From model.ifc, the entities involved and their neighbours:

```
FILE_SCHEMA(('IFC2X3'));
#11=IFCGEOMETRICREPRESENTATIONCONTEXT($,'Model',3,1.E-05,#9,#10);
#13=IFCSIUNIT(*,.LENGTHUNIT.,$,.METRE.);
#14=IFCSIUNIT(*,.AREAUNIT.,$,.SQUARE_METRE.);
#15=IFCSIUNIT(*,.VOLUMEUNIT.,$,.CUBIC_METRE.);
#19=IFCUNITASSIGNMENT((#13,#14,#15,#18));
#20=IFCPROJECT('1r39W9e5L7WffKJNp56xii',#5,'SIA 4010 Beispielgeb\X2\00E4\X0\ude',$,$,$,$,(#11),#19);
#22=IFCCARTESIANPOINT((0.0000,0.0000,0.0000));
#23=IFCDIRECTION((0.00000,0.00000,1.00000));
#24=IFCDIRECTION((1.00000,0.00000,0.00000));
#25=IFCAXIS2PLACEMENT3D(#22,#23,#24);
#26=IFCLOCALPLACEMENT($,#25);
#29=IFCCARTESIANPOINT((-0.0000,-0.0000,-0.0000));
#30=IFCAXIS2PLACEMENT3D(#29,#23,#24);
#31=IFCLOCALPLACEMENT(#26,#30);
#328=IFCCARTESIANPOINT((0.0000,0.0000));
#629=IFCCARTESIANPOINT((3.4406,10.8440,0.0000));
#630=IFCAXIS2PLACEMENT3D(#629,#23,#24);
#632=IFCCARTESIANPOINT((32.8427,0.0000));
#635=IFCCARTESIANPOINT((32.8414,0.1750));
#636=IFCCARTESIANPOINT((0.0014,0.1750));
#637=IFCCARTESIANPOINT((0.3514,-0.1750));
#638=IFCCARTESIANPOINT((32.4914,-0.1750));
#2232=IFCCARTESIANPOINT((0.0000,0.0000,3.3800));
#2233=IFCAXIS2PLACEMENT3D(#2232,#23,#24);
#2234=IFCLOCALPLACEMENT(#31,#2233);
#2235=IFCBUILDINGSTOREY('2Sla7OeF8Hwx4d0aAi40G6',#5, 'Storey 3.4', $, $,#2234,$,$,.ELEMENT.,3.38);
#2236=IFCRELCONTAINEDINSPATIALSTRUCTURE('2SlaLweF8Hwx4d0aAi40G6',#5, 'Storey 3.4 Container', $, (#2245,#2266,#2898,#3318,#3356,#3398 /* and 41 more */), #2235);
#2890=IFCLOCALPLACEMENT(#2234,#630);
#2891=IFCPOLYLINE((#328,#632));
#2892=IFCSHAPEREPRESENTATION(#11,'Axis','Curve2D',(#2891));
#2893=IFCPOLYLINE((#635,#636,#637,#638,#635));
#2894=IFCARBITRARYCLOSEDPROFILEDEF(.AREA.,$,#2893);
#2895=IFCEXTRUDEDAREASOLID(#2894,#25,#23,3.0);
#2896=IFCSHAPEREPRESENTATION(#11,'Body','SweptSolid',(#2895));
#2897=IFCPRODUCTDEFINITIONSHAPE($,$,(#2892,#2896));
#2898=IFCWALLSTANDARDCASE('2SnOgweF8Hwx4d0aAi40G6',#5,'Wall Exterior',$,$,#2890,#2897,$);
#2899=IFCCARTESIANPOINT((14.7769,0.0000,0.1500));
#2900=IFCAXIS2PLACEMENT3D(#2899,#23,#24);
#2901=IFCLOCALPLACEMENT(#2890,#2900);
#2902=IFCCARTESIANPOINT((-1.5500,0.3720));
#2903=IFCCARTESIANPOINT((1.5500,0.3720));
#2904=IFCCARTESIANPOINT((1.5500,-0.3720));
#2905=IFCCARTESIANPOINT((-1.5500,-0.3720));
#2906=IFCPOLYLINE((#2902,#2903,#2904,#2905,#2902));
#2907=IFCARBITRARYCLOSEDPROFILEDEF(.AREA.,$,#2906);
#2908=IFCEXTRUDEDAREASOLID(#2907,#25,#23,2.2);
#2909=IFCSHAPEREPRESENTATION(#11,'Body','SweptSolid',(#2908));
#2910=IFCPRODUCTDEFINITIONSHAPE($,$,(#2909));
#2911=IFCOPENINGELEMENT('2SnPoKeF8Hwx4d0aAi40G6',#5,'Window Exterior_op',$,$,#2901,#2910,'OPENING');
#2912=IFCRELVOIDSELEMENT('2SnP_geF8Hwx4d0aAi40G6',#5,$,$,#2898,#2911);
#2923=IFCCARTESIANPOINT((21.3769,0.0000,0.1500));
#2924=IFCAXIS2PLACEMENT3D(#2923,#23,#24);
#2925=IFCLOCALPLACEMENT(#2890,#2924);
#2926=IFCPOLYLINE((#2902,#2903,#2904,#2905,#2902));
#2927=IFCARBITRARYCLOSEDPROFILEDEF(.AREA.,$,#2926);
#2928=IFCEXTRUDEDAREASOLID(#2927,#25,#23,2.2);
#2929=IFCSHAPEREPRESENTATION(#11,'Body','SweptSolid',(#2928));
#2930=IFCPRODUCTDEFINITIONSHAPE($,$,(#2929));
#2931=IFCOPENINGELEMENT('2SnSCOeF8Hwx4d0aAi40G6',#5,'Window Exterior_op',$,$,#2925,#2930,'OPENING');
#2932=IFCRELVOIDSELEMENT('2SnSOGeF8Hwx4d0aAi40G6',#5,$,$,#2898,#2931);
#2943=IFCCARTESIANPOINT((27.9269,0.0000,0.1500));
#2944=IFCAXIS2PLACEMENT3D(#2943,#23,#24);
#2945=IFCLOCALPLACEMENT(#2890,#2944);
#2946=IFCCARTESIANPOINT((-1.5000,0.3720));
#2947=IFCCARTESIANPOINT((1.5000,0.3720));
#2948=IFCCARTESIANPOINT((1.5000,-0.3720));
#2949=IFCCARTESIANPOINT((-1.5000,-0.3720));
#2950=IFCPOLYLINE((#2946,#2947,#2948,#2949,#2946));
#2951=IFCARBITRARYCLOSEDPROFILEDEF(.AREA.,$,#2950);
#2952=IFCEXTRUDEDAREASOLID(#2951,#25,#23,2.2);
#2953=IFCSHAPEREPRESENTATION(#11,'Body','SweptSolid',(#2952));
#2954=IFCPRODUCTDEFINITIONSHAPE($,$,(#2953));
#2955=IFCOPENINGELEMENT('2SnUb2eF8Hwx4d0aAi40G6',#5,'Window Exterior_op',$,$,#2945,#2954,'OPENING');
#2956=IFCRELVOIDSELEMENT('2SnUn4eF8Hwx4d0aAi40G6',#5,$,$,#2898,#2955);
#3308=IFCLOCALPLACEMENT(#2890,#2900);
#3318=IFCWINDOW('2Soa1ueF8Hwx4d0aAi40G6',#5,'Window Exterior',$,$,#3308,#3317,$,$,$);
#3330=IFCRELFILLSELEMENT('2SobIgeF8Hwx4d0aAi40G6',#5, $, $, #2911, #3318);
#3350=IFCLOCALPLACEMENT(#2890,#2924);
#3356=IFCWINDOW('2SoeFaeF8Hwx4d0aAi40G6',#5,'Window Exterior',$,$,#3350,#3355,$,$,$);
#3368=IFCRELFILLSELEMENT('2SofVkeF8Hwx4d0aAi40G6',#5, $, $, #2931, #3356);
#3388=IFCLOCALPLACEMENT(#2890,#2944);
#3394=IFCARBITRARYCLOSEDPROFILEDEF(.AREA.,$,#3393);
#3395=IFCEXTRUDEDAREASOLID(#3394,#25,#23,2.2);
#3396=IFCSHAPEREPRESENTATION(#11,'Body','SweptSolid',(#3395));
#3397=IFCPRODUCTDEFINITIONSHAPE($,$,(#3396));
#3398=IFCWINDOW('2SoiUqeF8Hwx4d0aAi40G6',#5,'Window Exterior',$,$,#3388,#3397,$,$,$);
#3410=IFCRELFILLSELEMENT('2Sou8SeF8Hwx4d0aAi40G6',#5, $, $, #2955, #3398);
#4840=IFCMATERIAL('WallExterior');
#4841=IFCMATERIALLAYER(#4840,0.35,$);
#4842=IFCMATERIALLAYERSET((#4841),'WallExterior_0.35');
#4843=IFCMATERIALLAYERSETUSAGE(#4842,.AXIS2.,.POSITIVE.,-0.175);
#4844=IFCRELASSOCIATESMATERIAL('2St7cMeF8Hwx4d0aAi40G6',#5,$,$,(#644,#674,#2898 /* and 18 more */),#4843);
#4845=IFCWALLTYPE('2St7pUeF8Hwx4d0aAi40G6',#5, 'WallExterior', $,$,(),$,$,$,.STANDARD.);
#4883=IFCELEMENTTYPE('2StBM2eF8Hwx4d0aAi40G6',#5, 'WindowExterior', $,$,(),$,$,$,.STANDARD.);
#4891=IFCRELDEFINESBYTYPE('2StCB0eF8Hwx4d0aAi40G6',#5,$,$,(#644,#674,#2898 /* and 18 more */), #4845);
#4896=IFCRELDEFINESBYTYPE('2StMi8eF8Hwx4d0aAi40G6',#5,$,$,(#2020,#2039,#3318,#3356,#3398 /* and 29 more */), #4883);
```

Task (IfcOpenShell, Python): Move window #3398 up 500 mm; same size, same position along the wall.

```python
import numpy as np
import ifcopenshell
import ifcopenshell.api.geometry
import ifcopenshell.util.placement
import ifcopenshell.util.unit

model = ifcopenshell.open("model.ifc")
unit_scale = ifcopenshell.util.unit.calculate_unit_scale(model)

window = model.by_guid("2SoiUqeF8Hwx4d0aAi40G6")
opening = window.FillsVoids[0].RelatingOpeningElement
dz = 0.5 / unit_scale

shift = np.array([0.0, 0.0, dz])
# The window is not placed relative to its opening, so move both.
for product in (opening, window):
    matrix = ifcopenshell.util.placement.get_local_placement(product.ObjectPlacement)
    matrix[:3, 3] += shift
    ifcopenshell.api.geometry.edit_object_placement(model, product=product, matrix=matrix, is_si=False)

print(f"moved by {dz * unit_scale:+.3f} m")

model.write("model_v2.ifc")
```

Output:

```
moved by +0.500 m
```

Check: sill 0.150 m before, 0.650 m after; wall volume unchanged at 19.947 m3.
